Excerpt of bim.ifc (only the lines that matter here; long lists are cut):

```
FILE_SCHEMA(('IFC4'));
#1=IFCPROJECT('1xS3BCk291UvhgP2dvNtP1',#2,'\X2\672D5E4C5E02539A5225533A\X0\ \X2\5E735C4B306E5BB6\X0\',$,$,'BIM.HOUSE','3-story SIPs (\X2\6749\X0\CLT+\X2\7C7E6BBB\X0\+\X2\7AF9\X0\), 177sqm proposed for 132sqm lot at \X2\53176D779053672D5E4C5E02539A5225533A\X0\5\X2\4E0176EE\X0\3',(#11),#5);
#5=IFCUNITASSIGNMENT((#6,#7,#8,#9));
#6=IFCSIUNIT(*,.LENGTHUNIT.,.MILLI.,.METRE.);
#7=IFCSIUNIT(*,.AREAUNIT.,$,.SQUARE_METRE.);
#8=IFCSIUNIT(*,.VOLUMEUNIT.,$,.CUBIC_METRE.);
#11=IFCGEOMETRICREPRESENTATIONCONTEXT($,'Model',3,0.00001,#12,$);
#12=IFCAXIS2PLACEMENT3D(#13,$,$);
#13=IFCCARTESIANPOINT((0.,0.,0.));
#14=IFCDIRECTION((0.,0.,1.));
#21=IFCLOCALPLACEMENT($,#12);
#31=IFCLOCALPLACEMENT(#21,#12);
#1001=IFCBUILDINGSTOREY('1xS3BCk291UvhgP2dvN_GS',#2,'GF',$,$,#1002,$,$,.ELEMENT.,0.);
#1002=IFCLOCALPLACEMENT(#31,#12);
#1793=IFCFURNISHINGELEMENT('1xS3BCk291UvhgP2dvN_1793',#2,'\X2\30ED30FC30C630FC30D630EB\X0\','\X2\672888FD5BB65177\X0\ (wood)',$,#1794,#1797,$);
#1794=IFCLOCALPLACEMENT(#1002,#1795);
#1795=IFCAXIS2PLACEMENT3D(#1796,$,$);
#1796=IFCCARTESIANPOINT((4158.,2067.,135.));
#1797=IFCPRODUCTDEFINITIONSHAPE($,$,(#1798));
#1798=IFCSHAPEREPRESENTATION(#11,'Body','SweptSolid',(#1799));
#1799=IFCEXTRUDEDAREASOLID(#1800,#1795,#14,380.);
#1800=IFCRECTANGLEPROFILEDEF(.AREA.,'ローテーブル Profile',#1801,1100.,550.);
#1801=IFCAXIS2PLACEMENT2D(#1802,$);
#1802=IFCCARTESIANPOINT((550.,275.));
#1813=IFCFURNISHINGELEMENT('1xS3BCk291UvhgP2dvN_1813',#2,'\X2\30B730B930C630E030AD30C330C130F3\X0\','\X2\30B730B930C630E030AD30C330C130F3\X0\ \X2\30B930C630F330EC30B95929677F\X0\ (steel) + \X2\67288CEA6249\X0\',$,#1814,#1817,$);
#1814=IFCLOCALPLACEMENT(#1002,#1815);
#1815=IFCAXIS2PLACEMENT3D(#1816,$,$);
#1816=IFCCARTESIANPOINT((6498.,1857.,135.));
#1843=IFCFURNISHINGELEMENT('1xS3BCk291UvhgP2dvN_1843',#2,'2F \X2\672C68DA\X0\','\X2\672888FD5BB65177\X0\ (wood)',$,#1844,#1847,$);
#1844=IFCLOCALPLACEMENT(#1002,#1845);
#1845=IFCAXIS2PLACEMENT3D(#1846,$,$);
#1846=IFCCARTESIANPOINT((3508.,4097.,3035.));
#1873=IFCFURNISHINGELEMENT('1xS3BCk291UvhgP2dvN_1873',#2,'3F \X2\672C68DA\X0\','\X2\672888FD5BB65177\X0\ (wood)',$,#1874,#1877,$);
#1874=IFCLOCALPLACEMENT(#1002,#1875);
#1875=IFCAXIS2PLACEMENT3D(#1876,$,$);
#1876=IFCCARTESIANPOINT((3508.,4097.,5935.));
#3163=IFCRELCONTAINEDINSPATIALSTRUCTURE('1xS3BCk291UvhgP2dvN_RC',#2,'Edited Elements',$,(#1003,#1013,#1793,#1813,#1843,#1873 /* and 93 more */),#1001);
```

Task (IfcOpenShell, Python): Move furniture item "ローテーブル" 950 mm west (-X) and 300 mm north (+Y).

```python
import ifcopenshell
import ifcopenshell.api.geometry
import ifcopenshell.util.placement

model = ifcopenshell.open("bim.ifc")

item = model.by_id(1793)
matrix = ifcopenshell.util.placement.get_local_placement(item.ObjectPlacement)
matrix[0, 3] -= 950.0
matrix[1, 3] += 300.0
ifcopenshell.api.geometry.edit_object_placement(model, product=item, matrix=matrix, is_si=False)

print(ifcopenshell.util.placement.get_local_placement(item.ObjectPlacement).round(3) + 0.0)

model.write("bim_edited.ifc")
```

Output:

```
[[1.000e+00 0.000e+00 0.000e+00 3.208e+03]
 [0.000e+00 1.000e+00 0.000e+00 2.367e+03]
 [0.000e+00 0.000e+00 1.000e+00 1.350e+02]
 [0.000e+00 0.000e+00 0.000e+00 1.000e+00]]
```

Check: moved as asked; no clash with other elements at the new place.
